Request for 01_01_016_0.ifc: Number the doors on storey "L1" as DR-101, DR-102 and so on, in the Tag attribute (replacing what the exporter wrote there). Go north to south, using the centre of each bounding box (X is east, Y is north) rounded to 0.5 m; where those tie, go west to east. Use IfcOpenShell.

First a look at what the model holds.

```python
import ifcopenshell
import ifcopenshell.util.element
import ifcopenshell.util.placement

model = ifcopenshell.open("01_01_016_0.ifc")
print(model.schema)
storey = next(s for s in model.by_type("IfcBuildingStorey") if s.Name == "L1")
doors = [e for e in ifcopenshell.util.element.get_decomposition(storey) if e.is_a("IfcDoor")]
for e in sorted(doors, key=lambda e: e.id()):
    origin = ifcopenshell.util.placement.get_local_placement(e.ObjectPlacement)[:3, 3]
    print(e.id(), e.Tag, e.Name, origin.round(2) + 0.0, sep=" | ")
```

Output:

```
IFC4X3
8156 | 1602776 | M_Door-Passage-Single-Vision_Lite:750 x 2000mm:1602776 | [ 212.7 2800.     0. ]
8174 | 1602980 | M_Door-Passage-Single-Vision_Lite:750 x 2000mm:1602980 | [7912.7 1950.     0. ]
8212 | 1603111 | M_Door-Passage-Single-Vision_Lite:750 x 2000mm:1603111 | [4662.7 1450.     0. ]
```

```python
import ifcopenshell
import ifcopenshell.geom
import ifcopenshell.util.element
import ifcopenshell.util.shape

model = ifcopenshell.open("01_01_016_0.ifc")
settings = ifcopenshell.geom.settings()
settings.set("use-world-coords", True)


def centre(element):
    shape = ifcopenshell.geom.create_shape(settings, element)
    return ifcopenshell.util.shape.get_bbox_centroid(shape.geometry)


storey = next(s for s in model.by_type("IfcBuildingStorey") if s.Name == "L1")
doors = [e for e in ifcopenshell.util.element.get_decomposition(storey) if e.is_a("IfcDoor")]

# Insertion points can sit at a corner or the storey origin, so sort by the geometry (in metres).
centres = {e: centre(e) for e in doors}
doors.sort(key=lambda e: (-round(centres[e][1] / 0.5), centres[e][0]))

for i, e in enumerate(doors, start=1):
    number = f"DR-1{i:02d}"
    e.Tag = number
    print(e.id(), number)

model.write("01_01_016_0_v2.ifc")
```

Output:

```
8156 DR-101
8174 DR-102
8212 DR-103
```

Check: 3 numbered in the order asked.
